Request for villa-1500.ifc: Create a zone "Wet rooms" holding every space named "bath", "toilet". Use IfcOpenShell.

First a look at what the model holds.

```python
import ifcopenshell

model = ifcopenshell.open("villa-1500.ifc")
print(model.schema)
seen = {}
for space in model.by_type("IfcSpace"):
    seen[space.LongName] = seen.get(space.LongName, 0) + 1
for name, count in sorted(seen.items(), key=str):
    print(count, "x", name)
print("zones:", [z.Name for z in model.by_type("IfcZone")][:20])
```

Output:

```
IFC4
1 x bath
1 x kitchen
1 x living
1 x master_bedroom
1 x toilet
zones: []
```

```python
import ifcopenshell
import ifcopenshell.api.group
import ifcopenshell.api.root

model = ifcopenshell.open("villa-1500.ifc")

names = {"bath", "toilet"}
spaces = [s for s in model.by_type("IfcSpace") if s.LongName in names]

zone = ifcopenshell.api.root.create_entity(model, ifc_class="IfcZone", name="Wet rooms")
ifcopenshell.api.group.assign_group(model, products=spaces, group=zone)
print(len(spaces), "spaces in", zone.Name)

model.write("villa-1500-out.ifc")
```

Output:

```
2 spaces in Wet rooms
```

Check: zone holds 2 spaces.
